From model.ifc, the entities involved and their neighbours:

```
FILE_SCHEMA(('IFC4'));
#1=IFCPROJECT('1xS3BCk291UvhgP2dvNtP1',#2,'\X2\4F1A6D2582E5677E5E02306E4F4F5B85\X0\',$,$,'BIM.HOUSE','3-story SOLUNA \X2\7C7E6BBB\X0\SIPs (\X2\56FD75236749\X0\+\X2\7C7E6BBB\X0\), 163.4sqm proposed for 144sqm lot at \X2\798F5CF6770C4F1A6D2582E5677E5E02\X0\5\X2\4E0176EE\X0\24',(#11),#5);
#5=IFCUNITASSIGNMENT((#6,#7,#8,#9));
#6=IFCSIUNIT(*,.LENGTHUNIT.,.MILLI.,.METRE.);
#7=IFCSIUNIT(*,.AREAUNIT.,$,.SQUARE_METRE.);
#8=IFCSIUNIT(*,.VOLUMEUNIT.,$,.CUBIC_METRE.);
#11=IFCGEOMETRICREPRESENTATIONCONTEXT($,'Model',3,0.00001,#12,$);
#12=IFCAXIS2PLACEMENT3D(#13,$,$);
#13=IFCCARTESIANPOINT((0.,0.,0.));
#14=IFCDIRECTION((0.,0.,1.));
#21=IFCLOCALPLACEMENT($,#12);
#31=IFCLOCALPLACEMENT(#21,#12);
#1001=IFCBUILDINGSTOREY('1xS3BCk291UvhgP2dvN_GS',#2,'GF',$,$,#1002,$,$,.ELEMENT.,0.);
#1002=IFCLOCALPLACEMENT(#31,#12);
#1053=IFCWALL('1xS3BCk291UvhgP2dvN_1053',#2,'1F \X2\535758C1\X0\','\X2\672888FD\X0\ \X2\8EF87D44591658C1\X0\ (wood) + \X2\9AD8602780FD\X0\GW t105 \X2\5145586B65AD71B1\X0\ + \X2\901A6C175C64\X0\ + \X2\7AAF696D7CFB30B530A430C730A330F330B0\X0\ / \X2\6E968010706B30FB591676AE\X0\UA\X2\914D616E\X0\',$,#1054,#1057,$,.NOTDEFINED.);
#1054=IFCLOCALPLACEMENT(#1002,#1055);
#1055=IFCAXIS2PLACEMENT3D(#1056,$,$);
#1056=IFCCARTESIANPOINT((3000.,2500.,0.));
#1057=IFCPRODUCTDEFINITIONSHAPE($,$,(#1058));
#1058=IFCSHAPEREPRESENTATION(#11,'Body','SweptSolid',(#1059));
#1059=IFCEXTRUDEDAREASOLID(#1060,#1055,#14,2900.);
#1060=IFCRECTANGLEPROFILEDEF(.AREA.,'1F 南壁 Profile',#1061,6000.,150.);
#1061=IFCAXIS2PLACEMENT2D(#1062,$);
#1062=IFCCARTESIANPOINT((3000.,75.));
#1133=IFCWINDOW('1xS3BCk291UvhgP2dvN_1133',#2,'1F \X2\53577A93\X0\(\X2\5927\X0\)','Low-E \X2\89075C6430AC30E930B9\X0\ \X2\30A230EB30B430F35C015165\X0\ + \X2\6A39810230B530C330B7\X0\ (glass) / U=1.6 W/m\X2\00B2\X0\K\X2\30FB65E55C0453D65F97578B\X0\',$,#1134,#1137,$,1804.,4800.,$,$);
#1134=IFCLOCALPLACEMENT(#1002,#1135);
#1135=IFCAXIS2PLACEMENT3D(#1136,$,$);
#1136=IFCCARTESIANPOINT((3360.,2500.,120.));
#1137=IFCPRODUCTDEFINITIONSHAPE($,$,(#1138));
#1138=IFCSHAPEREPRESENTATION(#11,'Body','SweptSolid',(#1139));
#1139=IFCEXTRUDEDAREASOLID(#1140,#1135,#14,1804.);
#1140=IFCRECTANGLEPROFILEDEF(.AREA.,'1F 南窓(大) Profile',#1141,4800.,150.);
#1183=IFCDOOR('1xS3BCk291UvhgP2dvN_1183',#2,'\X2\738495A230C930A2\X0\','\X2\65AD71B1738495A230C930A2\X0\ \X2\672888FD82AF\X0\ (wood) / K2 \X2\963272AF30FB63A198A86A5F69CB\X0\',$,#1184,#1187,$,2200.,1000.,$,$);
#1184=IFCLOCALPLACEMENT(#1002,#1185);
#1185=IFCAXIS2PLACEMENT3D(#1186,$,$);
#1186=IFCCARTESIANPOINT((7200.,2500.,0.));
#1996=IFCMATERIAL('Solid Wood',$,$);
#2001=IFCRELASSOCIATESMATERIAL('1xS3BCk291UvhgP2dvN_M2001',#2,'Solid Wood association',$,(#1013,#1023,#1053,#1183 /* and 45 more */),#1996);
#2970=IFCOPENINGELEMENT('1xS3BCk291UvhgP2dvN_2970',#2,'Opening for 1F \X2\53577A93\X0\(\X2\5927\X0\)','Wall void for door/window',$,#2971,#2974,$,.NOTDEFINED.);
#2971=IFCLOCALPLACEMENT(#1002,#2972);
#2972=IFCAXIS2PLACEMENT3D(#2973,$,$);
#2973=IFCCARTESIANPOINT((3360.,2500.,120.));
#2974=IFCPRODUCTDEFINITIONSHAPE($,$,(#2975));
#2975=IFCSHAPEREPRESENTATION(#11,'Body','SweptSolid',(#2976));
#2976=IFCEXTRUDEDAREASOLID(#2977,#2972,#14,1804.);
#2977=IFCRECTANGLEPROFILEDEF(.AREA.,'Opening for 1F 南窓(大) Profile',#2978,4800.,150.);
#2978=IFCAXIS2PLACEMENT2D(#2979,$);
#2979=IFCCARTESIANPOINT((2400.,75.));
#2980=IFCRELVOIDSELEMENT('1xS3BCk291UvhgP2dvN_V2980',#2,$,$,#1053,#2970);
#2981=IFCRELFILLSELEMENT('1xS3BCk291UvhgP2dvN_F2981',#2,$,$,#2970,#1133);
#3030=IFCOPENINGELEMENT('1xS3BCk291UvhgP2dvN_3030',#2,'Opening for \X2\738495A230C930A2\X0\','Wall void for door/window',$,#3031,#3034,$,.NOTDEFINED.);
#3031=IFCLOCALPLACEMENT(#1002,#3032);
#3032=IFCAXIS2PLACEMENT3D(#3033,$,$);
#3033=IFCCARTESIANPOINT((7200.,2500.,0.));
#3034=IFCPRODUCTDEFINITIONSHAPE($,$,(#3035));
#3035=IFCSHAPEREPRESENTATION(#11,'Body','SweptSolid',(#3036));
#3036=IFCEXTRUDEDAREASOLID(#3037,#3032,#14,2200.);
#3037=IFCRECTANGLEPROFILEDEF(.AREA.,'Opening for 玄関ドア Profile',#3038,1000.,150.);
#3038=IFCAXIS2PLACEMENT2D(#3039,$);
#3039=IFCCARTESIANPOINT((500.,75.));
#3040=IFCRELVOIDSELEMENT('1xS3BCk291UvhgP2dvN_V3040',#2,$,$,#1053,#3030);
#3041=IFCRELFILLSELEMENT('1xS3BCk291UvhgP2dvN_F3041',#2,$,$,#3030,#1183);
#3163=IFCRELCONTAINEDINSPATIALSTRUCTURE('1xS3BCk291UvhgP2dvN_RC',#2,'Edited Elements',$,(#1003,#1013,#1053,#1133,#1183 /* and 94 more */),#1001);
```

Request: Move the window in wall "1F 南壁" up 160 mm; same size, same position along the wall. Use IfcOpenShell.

```python
import numpy as np
import ifcopenshell
import ifcopenshell.api.geometry
import ifcopenshell.util.placement
import ifcopenshell.util.unit

model = ifcopenshell.open("model.ifc")
unit_scale = ifcopenshell.util.unit.calculate_unit_scale(model)

window = model.by_guid("1xS3BCk291UvhgP2dvN_1133")
opening = window.FillsVoids[0].RelatingOpeningElement
dz = 0.16 / unit_scale

shift = np.array([0.0, 0.0, dz])
# The window is not placed relative to its opening, so move both.
for product in (opening, window):
    matrix = ifcopenshell.util.placement.get_local_placement(product.ObjectPlacement)
    matrix[:3, 3] += shift
    ifcopenshell.api.geometry.edit_object_placement(model, product=product, matrix=matrix, is_si=False)

print(f"moved by {dz * unit_scale:+.3f} m")

model.write("model_updated.ifc")
```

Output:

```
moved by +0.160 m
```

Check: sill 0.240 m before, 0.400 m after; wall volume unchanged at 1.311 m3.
